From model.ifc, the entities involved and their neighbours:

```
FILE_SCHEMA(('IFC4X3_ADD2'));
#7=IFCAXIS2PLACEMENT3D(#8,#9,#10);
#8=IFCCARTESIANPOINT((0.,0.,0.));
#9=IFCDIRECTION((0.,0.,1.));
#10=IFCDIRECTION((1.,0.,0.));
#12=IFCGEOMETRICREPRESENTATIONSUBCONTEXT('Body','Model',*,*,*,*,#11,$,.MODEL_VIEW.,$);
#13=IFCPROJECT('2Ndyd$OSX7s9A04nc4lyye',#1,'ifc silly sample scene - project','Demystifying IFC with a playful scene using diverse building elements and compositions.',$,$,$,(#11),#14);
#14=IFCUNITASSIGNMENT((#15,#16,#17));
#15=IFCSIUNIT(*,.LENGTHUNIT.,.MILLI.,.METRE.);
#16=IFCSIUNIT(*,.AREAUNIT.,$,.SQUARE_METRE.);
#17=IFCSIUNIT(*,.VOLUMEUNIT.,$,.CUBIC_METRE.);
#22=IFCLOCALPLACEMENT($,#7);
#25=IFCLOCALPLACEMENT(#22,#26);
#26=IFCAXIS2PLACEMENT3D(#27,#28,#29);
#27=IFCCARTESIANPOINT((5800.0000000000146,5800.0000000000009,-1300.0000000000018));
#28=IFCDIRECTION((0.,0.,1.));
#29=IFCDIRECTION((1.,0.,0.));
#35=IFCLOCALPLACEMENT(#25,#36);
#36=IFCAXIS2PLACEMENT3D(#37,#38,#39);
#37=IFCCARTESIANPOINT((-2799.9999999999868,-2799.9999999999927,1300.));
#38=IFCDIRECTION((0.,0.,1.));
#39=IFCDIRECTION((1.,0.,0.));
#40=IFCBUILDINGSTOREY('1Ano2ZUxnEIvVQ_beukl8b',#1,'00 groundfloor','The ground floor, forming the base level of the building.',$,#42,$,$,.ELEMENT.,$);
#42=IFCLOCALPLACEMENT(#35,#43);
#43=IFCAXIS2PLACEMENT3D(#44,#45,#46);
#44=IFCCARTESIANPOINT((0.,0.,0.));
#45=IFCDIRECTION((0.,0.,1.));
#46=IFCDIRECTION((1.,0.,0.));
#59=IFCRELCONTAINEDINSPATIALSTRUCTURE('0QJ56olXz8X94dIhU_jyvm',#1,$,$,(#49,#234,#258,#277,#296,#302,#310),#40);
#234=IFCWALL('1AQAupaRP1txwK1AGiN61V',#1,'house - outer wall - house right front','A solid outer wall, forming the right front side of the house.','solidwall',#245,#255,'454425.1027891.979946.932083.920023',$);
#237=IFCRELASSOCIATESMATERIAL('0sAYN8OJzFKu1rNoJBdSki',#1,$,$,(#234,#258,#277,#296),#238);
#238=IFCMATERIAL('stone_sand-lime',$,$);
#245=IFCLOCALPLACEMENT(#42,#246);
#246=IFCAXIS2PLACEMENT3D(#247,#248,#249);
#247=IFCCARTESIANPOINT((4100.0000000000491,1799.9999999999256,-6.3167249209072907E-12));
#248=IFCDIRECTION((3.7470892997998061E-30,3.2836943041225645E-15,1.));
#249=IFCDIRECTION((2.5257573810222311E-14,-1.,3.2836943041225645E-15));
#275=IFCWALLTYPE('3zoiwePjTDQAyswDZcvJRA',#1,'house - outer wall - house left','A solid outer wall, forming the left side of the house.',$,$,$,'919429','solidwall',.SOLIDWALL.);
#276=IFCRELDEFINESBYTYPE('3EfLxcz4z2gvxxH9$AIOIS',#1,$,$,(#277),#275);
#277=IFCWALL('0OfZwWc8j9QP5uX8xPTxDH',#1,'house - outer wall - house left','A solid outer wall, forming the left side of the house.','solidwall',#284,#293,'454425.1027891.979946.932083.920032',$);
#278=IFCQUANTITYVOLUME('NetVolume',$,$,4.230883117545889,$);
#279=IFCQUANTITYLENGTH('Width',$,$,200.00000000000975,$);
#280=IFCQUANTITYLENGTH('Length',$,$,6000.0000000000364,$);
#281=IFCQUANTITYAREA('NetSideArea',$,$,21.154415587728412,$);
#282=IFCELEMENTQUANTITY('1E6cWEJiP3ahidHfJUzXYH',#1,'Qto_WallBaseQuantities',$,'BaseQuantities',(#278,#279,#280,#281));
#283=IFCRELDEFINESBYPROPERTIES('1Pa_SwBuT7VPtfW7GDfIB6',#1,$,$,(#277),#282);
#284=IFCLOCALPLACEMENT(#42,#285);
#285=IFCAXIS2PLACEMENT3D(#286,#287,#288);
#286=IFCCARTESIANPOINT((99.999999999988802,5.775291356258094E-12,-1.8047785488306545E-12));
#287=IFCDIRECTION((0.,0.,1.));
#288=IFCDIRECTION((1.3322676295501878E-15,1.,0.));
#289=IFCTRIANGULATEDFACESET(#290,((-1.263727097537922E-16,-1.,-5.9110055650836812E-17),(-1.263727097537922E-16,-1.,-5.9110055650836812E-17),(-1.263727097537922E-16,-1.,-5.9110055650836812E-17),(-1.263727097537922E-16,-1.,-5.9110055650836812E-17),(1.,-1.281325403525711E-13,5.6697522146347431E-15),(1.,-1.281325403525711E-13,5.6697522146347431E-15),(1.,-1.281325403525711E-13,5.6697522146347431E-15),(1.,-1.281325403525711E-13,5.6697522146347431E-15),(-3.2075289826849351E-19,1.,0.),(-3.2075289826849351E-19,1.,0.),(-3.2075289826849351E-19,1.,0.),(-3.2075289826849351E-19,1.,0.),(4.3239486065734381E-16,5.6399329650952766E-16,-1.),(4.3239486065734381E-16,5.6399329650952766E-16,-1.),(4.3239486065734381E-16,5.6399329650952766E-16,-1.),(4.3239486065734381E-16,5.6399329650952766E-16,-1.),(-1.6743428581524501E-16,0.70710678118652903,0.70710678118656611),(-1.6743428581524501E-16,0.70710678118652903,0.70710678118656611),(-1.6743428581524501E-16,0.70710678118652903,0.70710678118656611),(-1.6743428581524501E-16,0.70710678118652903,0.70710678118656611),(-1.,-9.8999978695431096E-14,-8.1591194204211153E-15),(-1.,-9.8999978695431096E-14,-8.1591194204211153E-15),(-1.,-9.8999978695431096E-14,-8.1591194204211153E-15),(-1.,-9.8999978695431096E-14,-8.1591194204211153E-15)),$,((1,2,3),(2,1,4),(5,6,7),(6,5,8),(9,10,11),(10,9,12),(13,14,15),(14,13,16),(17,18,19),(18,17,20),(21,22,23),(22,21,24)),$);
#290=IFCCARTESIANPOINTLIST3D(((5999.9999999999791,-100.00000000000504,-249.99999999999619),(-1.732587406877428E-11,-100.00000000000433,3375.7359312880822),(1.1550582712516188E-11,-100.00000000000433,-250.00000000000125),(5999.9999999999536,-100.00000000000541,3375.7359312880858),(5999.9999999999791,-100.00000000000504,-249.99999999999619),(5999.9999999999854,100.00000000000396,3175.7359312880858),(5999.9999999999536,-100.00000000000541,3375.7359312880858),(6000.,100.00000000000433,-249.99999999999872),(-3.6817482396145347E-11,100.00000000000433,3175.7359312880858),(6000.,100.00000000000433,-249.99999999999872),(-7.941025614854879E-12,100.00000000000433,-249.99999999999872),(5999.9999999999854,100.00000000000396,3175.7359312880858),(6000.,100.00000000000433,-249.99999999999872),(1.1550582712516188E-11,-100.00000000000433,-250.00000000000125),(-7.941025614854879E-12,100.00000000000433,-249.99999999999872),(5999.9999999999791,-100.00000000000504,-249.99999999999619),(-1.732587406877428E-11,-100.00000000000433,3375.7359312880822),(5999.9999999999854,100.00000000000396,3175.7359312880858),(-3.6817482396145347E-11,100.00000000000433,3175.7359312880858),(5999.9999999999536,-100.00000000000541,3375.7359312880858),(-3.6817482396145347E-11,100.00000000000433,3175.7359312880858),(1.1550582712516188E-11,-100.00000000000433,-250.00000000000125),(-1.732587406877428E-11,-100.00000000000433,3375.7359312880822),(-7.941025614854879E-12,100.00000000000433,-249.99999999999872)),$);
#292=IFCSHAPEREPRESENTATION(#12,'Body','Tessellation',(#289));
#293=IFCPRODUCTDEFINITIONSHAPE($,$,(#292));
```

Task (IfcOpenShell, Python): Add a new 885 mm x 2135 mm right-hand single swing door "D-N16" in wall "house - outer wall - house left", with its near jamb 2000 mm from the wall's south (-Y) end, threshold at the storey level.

```python
import numpy as np
import ifcopenshell
import ifcopenshell.api.feature
import ifcopenshell.api.geometry
import ifcopenshell.api.pset
import ifcopenshell.api.root
import ifcopenshell.api.spatial
import ifcopenshell.geom
import ifcopenshell.util.element
import ifcopenshell.util.placement
import ifcopenshell.util.representation
import ifcopenshell.util.shape
import ifcopenshell.util.unit

model = ifcopenshell.open("model.ifc")
unit_scale = ifcopenshell.util.unit.calculate_unit_scale(model)
area_scale = ifcopenshell.util.unit.calculate_unit_scale(model, "AREAUNIT")
volume_scale = ifcopenshell.util.unit.calculate_unit_scale(model, "VOLUMEUNIT")
settings = ifcopenshell.geom.settings()


def volume(element):
    """Net volume in cubic metres, openings subtracted."""
    shape = ifcopenshell.geom.create_shape(settings, element)
    return ifcopenshell.util.shape.get_volume(shape.geometry)


wall = model.by_guid("0OfZwWc8j9QP5uX8xPTxDH")
storey = ifcopenshell.util.element.get_container(wall, ifc_class="IfcBuildingStorey")
context = ifcopenshell.util.representation.get_context(model, "Model", "Body", "MODEL_VIEW")
before = volume(wall)

width, height, from_end, sill = 0.885, 2.135, 2, 0.0  # metres

# The wall runs along its own X axis, and the end named is its -X end.
wall_shape = ifcopenshell.geom.create_shape(settings, wall)
x, y, z = ifcopenshell.util.shape.get_vertices(wall_shape.geometry).T
start = x.min() + from_end
face, thickness = float(y.min()), float(y.max() - y.min())
wall_matrix = ifcopenshell.util.placement.get_local_placement(wall.ObjectPlacement)
level = ifcopenshell.util.placement.get_local_placement(storey.ObjectPlacement)[2, 3]


def in_wall(x, y):
    """Placement at x, y metres in the wall's axes, at sill height."""
    matrix = wall_matrix.copy()
    matrix[:, 3] = wall_matrix @ np.array([x / unit_scale, y / unit_scale, 0.0, 1.0])
    matrix[2, 3] = level + sill / unit_scale
    return matrix


# Opening: a box that overshoots both wall faces by 50 mm.
opening = ifcopenshell.api.root.create_entity(model, ifc_class="IfcOpeningElement", predefined_type="OPENING")
box = ifcopenshell.api.geometry.add_wall_representation(
    model, context=context, length=width, height=height, thickness=thickness + 0.1
)
ifcopenshell.api.geometry.assign_representation(model, product=opening, representation=box)
ifcopenshell.api.geometry.edit_object_placement(model, product=opening, matrix=in_wall(start, face - 0.05), is_si=False)
ifcopenshell.api.feature.add_feature(model, feature=opening, element=wall)

door = ifcopenshell.api.root.create_entity(model, ifc_class="IfcDoor", name="D-N16", predefined_type="DOOR")
door.OverallWidth, door.OverallHeight = width / unit_scale, height / unit_scale
door.OperationType = "SINGLE_SWING_RIGHT"
body = ifcopenshell.api.geometry.add_door_representation(
    model,
    context=context,
    overall_width=door.OverallWidth,
    overall_height=door.OverallHeight,
    operation_type="SINGLE_SWING_RIGHT",
    lining_properties={"LiningDepth": thickness / unit_scale, "ThresholdDepth": thickness / unit_scale},
)
ifcopenshell.api.geometry.assign_representation(model, product=door, representation=body)
ifcopenshell.api.spatial.assign_container(model, products=[door], relating_structure=storey)
ifcopenshell.api.feature.add_filling(model, opening=opening, element=door)

# The lining spans the wall, so the door starts at the wall face.
ifcopenshell.api.geometry.edit_object_placement(model, product=door, matrix=in_wall(start, face), is_si=False)

after = volume(wall)

# Update the wall's stored quantities.
qto = model.by_id(ifcopenshell.util.element.get_pset(wall, "Qto_WallBaseQuantities", should_inherit=False)["id"])
ifcopenshell.api.pset.edit_qto(model, qto=qto, properties={
    "NetVolume": after / volume_scale,
    "NetSideArea": after / thickness / area_scale,
})

print(f"wall volume {before:.3f} -> {after:.3f} m3")

model.write("model_updated.ifc")
```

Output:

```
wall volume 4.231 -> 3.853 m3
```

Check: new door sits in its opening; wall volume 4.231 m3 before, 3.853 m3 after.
